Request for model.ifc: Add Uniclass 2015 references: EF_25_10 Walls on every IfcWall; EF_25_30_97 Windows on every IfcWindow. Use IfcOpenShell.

First a look at what the model holds.

```python
import ifcopenshell

model = ifcopenshell.open("model.ifc")
print(model.schema)
print("classifications:", [c.Name for c in model.by_type("IfcClassification")])
for ifc_class in ("IfcDoor", "IfcRoof", "IfcStair", "IfcWall", "IfcWindow"):
    print(ifc_class, len(model.by_type(ifc_class)))
```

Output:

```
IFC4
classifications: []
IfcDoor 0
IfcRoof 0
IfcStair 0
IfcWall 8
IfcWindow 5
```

```python
import ifcopenshell
import ifcopenshell.api.classification

model = ifcopenshell.open("model.ifc")

system = ifcopenshell.api.classification.add_classification(model, classification="Uniclass 2015")

codes = {
    "IfcWall": ("EF_25_10", "Walls"),
    "IfcWindow": ("EF_25_30_97", "Windows"),
}
for ifc_class, (code, name) in codes.items():
    products = model.by_type(ifc_class)
    ifcopenshell.api.classification.add_reference(
        model, products=products, classification=system, identification=code, name=name
    )
    print(code, len(products))

model.write("model_v2.ifc")
```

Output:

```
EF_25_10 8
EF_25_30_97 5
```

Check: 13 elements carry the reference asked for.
